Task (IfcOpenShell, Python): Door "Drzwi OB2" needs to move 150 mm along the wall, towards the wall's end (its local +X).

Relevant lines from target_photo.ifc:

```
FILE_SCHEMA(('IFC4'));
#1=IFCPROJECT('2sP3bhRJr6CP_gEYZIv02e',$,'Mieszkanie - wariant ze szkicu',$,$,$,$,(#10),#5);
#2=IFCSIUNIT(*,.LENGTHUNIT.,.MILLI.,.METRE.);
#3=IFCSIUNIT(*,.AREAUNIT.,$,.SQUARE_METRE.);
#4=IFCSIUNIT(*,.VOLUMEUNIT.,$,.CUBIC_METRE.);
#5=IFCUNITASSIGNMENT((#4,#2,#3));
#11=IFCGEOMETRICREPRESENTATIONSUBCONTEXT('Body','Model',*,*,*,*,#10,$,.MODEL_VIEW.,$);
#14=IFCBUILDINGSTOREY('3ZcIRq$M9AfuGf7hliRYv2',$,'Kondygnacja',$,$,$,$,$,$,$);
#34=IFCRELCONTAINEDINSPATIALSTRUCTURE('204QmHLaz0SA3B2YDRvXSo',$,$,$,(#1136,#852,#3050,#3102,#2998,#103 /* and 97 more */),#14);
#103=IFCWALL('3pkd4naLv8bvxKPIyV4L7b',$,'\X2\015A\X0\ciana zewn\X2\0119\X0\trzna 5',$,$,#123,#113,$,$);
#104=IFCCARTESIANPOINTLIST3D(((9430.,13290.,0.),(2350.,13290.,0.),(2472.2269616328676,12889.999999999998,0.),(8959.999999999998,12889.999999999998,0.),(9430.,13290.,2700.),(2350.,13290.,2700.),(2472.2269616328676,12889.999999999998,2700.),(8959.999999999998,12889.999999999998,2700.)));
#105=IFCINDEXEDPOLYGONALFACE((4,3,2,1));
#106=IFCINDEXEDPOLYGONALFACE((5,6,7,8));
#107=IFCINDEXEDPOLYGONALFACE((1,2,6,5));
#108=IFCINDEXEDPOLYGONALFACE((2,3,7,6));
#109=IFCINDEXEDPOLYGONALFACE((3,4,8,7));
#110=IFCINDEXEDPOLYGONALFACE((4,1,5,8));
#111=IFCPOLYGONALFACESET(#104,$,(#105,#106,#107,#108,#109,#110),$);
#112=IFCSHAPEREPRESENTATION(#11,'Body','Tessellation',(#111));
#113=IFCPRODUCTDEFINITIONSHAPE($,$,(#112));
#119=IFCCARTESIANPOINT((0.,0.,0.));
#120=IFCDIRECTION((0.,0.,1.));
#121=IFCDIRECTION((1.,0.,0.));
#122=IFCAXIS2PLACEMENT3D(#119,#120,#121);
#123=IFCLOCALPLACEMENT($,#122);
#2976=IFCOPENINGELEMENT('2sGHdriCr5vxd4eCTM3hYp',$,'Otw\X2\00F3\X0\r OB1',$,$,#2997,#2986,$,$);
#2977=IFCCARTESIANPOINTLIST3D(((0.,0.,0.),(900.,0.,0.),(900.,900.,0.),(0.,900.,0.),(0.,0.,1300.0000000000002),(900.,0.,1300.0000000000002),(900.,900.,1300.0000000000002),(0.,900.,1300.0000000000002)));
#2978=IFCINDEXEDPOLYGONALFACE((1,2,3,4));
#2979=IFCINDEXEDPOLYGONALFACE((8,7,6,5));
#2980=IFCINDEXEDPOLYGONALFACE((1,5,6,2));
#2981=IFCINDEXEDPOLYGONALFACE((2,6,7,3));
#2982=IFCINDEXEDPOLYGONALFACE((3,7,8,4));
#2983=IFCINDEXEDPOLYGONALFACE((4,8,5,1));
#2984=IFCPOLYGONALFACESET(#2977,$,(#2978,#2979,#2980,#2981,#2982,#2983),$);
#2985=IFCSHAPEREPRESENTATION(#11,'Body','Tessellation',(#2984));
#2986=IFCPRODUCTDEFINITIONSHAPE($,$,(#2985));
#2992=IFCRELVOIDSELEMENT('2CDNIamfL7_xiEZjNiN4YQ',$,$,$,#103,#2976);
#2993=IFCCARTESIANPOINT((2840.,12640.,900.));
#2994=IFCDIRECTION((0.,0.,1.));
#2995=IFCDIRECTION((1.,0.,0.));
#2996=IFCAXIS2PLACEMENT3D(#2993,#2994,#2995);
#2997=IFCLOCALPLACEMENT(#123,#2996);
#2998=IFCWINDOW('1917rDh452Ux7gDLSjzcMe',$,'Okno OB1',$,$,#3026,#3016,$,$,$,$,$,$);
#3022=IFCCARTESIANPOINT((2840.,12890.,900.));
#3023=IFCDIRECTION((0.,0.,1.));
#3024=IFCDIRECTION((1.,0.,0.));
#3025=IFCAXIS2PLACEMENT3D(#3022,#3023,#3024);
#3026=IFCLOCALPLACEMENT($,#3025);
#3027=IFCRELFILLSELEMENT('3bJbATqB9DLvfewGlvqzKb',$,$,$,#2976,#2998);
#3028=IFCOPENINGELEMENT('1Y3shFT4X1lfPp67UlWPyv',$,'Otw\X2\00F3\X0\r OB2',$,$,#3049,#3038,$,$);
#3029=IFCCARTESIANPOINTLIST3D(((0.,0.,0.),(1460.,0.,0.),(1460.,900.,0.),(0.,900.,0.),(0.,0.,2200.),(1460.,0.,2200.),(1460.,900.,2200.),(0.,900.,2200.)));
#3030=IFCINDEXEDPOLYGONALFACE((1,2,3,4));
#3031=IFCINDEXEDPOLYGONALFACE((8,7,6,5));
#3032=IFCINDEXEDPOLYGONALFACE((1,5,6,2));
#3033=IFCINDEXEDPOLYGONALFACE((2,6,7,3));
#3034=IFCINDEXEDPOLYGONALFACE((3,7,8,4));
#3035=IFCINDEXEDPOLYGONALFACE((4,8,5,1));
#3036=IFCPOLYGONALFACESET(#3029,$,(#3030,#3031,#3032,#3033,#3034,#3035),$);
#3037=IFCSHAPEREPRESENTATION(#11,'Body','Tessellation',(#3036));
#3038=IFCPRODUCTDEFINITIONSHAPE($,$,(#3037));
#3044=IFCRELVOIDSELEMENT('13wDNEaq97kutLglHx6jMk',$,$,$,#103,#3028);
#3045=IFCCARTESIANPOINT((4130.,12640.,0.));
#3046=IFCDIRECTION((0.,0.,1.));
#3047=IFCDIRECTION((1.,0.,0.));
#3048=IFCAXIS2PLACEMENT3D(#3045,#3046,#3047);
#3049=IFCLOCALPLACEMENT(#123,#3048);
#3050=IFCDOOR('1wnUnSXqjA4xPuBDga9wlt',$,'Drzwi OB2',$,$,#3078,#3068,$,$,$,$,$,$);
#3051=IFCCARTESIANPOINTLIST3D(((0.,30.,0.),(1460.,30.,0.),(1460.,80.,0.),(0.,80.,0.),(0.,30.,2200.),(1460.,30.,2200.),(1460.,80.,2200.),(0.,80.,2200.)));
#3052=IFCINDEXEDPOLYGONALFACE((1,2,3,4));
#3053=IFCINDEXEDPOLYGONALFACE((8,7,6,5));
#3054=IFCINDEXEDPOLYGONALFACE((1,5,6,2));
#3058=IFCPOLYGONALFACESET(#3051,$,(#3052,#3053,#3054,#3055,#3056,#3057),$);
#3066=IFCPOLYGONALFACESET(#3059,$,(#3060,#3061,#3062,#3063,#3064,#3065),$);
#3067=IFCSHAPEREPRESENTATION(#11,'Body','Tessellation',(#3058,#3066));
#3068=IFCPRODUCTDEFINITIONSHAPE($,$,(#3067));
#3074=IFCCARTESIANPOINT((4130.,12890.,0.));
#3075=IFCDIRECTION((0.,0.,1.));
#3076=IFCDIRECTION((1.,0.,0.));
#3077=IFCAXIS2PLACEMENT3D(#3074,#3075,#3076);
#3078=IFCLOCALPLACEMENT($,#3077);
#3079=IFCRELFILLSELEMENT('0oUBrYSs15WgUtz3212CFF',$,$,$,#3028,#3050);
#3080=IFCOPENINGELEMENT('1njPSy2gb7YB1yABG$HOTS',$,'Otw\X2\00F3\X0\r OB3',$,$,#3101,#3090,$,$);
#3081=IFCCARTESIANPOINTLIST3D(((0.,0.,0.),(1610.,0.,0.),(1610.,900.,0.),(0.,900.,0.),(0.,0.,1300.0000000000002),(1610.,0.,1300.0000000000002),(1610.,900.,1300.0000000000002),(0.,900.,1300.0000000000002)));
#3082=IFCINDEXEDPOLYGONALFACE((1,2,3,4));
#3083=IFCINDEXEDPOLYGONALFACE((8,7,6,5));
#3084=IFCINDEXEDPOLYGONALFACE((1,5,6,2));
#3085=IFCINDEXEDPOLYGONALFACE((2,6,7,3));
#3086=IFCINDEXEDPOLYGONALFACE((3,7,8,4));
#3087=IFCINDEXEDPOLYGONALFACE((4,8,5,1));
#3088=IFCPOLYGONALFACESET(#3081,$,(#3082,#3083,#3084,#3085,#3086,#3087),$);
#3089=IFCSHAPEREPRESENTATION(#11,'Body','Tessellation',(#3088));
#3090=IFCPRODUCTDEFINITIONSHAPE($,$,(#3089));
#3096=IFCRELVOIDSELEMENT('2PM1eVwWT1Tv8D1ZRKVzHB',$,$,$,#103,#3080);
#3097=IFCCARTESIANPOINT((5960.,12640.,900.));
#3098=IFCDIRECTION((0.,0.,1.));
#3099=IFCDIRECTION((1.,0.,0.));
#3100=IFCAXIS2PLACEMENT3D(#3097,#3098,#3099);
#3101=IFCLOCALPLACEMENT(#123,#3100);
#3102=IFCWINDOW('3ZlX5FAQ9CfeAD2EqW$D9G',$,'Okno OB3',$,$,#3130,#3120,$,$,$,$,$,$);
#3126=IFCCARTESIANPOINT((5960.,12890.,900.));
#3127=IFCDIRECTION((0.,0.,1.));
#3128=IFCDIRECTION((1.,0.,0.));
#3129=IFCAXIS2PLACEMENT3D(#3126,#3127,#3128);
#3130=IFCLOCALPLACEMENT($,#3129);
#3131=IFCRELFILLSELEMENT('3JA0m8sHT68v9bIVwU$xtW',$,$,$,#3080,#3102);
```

```python
import ifcopenshell
import ifcopenshell.api.geometry
import ifcopenshell.util.placement
import ifcopenshell.util.unit

model = ifcopenshell.open("target_photo.ifc")
unit_scale = ifcopenshell.util.unit.calculate_unit_scale(model)

door = model.by_id(3050)
opening = door.FillsVoids[0].RelatingOpeningElement
wall = opening.VoidsElements[0].RelatingBuildingElement

wall_matrix = ifcopenshell.util.placement.get_local_placement(wall.ObjectPlacement)
shift = wall_matrix[:3, 0] * 0.15 / unit_scale
before = ifcopenshell.util.placement.get_local_placement(door.ObjectPlacement)[:3, 3].copy()

# The door is not placed relative to its opening, so move both.
for product in (opening, door):
    matrix = ifcopenshell.util.placement.get_local_placement(product.ObjectPlacement)
    matrix[:3, 3] += shift
    ifcopenshell.api.geometry.edit_object_placement(model, product=product, matrix=matrix, is_si=False)

after = ifcopenshell.util.placement.get_local_placement(door.ObjectPlacement)[:3, 3]
print("door moved by", (after - before).round(3) + 0.0)

model.write("target_photo_edited.ifc")
```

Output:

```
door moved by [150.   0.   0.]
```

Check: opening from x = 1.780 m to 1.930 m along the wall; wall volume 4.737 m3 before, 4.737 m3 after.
